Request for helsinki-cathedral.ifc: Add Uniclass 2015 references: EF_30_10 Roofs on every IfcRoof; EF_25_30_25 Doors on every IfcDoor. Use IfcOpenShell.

First a look at what the model holds.

```python
import ifcopenshell

model = ifcopenshell.open("helsinki-cathedral.ifc")
print(model.schema)
print("classifications:", [c.Name for c in model.by_type("IfcClassification")])
for ifc_class in ("IfcDoor", "IfcRoof", "IfcStair", "IfcWall", "IfcWindow"):
    print(ifc_class, len(model.by_type(ifc_class)))
```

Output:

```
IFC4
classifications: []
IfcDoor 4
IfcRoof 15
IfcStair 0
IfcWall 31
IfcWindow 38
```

```python
import ifcopenshell
import ifcopenshell.api.classification

model = ifcopenshell.open("helsinki-cathedral.ifc")

system = ifcopenshell.api.classification.add_classification(model, classification="Uniclass 2015")

codes = {
    "IfcRoof": ("EF_30_10", "Roofs"),
    "IfcDoor": ("EF_25_30_25", "Doors"),
}
for ifc_class, (code, name) in codes.items():
    products = model.by_type(ifc_class)
    ifcopenshell.api.classification.add_reference(
        model, products=products, classification=system, identification=code, name=name
    )
    print(code, len(products))

model.write("helsinki-cathedral_updated.ifc")
```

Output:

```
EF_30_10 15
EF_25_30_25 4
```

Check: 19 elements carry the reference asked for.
